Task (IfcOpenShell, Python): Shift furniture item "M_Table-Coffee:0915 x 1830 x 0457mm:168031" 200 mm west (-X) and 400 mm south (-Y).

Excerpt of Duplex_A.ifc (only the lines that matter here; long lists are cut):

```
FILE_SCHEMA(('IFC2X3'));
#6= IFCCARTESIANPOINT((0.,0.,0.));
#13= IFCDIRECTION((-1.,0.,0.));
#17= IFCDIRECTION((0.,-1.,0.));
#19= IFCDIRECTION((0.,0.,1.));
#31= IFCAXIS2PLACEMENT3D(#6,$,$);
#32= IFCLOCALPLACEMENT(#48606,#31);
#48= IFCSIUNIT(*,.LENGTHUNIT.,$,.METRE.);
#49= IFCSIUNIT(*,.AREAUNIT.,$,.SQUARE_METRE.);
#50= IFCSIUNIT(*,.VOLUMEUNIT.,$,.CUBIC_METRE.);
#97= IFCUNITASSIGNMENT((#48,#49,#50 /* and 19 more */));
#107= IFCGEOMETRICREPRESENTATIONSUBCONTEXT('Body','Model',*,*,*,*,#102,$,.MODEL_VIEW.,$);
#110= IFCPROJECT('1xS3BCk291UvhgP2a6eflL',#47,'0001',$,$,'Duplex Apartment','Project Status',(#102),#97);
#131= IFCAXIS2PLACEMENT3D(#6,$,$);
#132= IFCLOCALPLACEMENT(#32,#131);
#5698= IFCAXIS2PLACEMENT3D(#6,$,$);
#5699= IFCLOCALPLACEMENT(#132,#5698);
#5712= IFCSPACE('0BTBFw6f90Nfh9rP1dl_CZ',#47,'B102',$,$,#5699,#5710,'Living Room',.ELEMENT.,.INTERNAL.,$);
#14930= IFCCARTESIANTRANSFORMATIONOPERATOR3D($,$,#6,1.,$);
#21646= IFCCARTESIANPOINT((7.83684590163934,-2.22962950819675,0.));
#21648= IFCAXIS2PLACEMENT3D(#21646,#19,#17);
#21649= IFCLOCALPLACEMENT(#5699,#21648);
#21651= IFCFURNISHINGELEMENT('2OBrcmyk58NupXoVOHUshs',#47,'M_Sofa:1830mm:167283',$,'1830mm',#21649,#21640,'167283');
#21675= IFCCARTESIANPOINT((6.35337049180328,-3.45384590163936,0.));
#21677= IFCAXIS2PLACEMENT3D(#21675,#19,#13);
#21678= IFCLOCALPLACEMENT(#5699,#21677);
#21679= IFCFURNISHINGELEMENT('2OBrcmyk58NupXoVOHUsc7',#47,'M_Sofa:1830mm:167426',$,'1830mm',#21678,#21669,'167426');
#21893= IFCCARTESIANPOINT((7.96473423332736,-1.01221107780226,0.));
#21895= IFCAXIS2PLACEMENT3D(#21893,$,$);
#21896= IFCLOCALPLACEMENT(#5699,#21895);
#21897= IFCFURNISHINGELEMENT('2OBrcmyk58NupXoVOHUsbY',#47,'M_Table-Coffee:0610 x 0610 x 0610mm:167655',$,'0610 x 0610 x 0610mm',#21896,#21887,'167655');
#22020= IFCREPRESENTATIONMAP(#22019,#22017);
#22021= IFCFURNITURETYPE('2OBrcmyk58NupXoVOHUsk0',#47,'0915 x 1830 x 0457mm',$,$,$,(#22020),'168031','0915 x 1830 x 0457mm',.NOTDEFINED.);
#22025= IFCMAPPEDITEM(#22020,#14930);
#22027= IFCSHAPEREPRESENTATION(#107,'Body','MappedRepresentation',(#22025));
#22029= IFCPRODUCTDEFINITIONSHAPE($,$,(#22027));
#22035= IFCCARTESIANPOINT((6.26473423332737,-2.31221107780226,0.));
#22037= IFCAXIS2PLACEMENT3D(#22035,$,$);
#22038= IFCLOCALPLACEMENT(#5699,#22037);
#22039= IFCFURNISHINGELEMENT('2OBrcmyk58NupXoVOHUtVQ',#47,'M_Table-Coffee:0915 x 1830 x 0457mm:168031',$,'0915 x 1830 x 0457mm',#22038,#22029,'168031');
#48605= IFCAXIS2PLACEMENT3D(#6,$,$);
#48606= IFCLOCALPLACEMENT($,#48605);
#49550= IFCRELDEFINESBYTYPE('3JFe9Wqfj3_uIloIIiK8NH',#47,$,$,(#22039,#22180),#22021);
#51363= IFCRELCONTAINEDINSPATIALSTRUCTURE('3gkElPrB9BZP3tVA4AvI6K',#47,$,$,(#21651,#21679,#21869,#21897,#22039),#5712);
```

```python
import ifcopenshell
import ifcopenshell.api.geometry
import ifcopenshell.util.placement
import ifcopenshell.util.unit

model = ifcopenshell.open("Duplex_A.ifc")
unit_scale = ifcopenshell.util.unit.calculate_unit_scale(model)

item = model.by_guid("2OBrcmyk58NupXoVOHUtVQ")
matrix = ifcopenshell.util.placement.get_local_placement(item.ObjectPlacement)
matrix[0, 3] -= 0.2 / unit_scale
matrix[1, 3] -= 0.4 / unit_scale
ifcopenshell.api.geometry.edit_object_placement(model, product=item, matrix=matrix, is_si=False)

print(ifcopenshell.util.placement.get_local_placement(item.ObjectPlacement).round(3) + 0.0)

model.write("Duplex_A_edited.ifc")
```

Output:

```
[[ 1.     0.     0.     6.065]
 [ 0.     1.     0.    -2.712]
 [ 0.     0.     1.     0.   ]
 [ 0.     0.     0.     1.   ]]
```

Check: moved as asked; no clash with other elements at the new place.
